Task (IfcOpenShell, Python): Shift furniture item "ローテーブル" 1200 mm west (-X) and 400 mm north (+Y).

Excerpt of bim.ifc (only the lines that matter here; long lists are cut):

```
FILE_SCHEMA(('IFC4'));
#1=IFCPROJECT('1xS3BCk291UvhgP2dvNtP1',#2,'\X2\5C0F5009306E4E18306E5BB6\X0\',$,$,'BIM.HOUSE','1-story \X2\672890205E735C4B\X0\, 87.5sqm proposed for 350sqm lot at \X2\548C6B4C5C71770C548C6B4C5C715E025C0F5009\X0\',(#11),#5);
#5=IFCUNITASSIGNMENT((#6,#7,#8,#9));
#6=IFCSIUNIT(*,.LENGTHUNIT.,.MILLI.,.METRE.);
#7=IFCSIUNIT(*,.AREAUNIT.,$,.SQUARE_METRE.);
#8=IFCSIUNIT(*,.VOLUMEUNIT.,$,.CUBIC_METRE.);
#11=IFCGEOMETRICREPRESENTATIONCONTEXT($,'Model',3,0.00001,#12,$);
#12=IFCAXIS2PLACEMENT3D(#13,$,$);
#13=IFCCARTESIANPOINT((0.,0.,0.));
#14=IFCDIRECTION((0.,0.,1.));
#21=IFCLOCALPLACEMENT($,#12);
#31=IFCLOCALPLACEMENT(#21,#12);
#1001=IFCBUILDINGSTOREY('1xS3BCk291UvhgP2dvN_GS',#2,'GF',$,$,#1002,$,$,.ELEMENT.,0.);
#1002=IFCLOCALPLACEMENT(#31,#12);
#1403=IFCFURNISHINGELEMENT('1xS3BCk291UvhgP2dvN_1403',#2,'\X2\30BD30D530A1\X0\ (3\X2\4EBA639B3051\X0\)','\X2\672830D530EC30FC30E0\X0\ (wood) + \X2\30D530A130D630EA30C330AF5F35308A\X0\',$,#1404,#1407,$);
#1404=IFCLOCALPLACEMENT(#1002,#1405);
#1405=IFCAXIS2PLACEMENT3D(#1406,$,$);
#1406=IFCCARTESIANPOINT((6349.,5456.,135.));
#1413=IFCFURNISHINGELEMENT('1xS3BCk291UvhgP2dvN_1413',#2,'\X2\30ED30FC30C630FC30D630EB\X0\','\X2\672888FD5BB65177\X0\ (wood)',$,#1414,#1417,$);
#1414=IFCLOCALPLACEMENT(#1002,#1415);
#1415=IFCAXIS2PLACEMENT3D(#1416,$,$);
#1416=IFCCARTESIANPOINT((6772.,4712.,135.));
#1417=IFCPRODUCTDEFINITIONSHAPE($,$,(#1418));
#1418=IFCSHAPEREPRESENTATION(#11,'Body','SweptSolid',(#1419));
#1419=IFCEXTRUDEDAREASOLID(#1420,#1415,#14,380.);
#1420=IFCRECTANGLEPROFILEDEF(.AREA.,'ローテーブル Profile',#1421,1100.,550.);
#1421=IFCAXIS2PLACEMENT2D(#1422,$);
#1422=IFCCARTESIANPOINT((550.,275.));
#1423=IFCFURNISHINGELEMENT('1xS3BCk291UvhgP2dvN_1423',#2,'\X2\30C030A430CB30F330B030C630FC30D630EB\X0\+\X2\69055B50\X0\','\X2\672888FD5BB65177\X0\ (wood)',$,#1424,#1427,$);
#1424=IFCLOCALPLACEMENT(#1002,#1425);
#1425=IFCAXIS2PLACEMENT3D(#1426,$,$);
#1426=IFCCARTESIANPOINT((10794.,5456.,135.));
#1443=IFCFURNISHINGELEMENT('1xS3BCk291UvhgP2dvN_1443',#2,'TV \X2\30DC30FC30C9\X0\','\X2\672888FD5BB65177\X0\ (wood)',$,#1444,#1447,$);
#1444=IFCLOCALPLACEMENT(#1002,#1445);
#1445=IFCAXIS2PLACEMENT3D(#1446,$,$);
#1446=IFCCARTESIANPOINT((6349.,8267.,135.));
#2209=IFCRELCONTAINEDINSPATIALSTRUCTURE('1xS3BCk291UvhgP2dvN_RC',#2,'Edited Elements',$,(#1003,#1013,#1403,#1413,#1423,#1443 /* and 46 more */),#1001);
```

```python
import ifcopenshell
import ifcopenshell.api.geometry
import ifcopenshell.util.placement

model = ifcopenshell.open("bim.ifc")

item = model.by_guid("1xS3BCk291UvhgP2dvN_1413")
matrix = ifcopenshell.util.placement.get_local_placement(item.ObjectPlacement)
matrix[0, 3] -= 1200.0
matrix[1, 3] += 400.0
ifcopenshell.api.geometry.edit_object_placement(model, product=item, matrix=matrix, is_si=False)

print(ifcopenshell.util.placement.get_local_placement(item.ObjectPlacement).round(3) + 0.0)

model.write("bim_v2.ifc")
```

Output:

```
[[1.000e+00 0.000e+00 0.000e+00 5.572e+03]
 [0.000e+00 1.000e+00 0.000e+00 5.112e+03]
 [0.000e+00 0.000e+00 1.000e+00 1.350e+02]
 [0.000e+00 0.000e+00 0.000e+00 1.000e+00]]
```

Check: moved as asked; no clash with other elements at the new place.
